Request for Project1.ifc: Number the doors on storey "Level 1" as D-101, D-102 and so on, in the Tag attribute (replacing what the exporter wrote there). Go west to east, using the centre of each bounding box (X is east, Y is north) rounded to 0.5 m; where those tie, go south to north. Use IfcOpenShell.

First a look at what the model holds.

```python
import ifcopenshell
import ifcopenshell.util.element
import ifcopenshell.util.placement

model = ifcopenshell.open("Project1.ifc")
print(model.schema)
storey = next(s for s in model.by_type("IfcBuildingStorey") if s.Name == "Level 1")
doors = [e for e in ifcopenshell.util.element.get_decomposition(storey) if e.is_a("IfcDoor")]
for e in sorted(doors, key=lambda e: e.id()):
    origin = ifcopenshell.util.placement.get_local_placement(e.ObjectPlacement)[:3, 3]
    print(e.id(), e.Tag, e.Name, origin.round(2) + 0.0, sep=" | ")
```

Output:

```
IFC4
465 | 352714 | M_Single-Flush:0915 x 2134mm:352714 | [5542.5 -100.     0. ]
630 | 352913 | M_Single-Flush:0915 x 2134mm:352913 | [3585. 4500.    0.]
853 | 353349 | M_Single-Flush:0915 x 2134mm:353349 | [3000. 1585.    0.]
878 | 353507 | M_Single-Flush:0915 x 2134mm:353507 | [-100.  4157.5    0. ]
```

```python
import ifcopenshell
import ifcopenshell.geom
import ifcopenshell.util.element
import ifcopenshell.util.shape

model = ifcopenshell.open("Project1.ifc")
settings = ifcopenshell.geom.settings()
settings.set("use-world-coords", True)


def centre(element):
    shape = ifcopenshell.geom.create_shape(settings, element)
    return ifcopenshell.util.shape.get_bbox_centroid(shape.geometry)


storey = next(s for s in model.by_type("IfcBuildingStorey") if s.Name == "Level 1")
doors = [e for e in ifcopenshell.util.element.get_decomposition(storey) if e.is_a("IfcDoor")]

# Insertion points can sit at a corner or the storey origin, so sort by the geometry (in metres).
centres = {e: centre(e) for e in doors}
doors.sort(key=lambda e: (round(centres[e][0] / 0.5), centres[e][1]))

for i, e in enumerate(doors, start=1):
    number = f"D-1{i:02d}"
    e.Tag = number
    print(e.id(), number)

model.write("Project1_edited.ifc")
```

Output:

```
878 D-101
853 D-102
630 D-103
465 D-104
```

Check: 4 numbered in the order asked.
